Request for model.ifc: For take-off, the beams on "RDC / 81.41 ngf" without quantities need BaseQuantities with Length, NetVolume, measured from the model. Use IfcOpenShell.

First a look at what the model holds.

```python
import ifcopenshell
import ifcopenshell.util.element
import ifcopenshell.util.unit

model = ifcopenshell.open("model.ifc")
print(model.schema)
for unit_type in ("LENGTHUNIT", "AREAUNIT", "VOLUMEUNIT"):
    print(unit_type, ifcopenshell.util.unit.calculate_unit_scale(model, unit_type))
storey = next(s for s in model.by_type("IfcBuildingStorey") if s.Name == "RDC / 81.41 ngf")
beams = [e for e in ifcopenshell.util.element.get_decomposition(storey) if e.is_a("IfcBeam")]
for e in sorted(beams, key=lambda e: e.id()):
    print(e.id(), e.is_a(), e.Name, list(ifcopenshell.util.element.get_psets(e, qtos_only=True)), sep=" | ")
```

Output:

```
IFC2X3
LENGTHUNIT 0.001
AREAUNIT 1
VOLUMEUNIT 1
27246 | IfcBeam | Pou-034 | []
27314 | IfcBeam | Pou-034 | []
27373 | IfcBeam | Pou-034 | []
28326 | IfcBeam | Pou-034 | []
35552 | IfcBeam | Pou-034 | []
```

```python
import ifcopenshell
import ifcopenshell.api.pset
import ifcopenshell.geom
import ifcopenshell.util.element
import ifcopenshell.util.shape
import ifcopenshell.util.unit

model = ifcopenshell.open("model.ifc")
unit_scale = ifcopenshell.util.unit.calculate_unit_scale(model)
volume_scale = ifcopenshell.util.unit.calculate_unit_scale(model, "VOLUMEUNIT")
settings = ifcopenshell.geom.settings()

storey = next(s for s in model.by_type("IfcBuildingStorey") if s.Name == "RDC / 81.41 ngf")
beams = [e for e in ifcopenshell.util.element.get_decomposition(storey) if e.is_a("IfcBeam")]

for e in sorted(beams, key=lambda e: e.id()):
    if ifcopenshell.util.element.get_psets(e, qtos_only=True, should_inherit=False):
        continue
    # Geometry comes back in metres, in the element's own axes.
    shape = ifcopenshell.geom.create_shape(settings, e)
    values = {
        "Length": ifcopenshell.util.shape.get_max_xyz(shape.geometry) / unit_scale,
        "NetVolume": ifcopenshell.util.shape.get_volume(shape.geometry) / volume_scale,
    }
    qto = ifcopenshell.api.pset.add_qto(model, product=e, name="BaseQuantities")
    ifcopenshell.api.pset.edit_qto(model, qto=qto, properties=values)
    print(e.id(), {k: round(v, 3) for k, v in values.items()})

model.write("model_rev.ifc")
```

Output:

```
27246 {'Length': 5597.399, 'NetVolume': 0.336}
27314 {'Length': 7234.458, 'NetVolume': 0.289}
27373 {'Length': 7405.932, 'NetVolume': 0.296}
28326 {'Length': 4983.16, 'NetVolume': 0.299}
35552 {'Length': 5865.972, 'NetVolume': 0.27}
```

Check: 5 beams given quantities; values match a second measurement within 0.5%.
